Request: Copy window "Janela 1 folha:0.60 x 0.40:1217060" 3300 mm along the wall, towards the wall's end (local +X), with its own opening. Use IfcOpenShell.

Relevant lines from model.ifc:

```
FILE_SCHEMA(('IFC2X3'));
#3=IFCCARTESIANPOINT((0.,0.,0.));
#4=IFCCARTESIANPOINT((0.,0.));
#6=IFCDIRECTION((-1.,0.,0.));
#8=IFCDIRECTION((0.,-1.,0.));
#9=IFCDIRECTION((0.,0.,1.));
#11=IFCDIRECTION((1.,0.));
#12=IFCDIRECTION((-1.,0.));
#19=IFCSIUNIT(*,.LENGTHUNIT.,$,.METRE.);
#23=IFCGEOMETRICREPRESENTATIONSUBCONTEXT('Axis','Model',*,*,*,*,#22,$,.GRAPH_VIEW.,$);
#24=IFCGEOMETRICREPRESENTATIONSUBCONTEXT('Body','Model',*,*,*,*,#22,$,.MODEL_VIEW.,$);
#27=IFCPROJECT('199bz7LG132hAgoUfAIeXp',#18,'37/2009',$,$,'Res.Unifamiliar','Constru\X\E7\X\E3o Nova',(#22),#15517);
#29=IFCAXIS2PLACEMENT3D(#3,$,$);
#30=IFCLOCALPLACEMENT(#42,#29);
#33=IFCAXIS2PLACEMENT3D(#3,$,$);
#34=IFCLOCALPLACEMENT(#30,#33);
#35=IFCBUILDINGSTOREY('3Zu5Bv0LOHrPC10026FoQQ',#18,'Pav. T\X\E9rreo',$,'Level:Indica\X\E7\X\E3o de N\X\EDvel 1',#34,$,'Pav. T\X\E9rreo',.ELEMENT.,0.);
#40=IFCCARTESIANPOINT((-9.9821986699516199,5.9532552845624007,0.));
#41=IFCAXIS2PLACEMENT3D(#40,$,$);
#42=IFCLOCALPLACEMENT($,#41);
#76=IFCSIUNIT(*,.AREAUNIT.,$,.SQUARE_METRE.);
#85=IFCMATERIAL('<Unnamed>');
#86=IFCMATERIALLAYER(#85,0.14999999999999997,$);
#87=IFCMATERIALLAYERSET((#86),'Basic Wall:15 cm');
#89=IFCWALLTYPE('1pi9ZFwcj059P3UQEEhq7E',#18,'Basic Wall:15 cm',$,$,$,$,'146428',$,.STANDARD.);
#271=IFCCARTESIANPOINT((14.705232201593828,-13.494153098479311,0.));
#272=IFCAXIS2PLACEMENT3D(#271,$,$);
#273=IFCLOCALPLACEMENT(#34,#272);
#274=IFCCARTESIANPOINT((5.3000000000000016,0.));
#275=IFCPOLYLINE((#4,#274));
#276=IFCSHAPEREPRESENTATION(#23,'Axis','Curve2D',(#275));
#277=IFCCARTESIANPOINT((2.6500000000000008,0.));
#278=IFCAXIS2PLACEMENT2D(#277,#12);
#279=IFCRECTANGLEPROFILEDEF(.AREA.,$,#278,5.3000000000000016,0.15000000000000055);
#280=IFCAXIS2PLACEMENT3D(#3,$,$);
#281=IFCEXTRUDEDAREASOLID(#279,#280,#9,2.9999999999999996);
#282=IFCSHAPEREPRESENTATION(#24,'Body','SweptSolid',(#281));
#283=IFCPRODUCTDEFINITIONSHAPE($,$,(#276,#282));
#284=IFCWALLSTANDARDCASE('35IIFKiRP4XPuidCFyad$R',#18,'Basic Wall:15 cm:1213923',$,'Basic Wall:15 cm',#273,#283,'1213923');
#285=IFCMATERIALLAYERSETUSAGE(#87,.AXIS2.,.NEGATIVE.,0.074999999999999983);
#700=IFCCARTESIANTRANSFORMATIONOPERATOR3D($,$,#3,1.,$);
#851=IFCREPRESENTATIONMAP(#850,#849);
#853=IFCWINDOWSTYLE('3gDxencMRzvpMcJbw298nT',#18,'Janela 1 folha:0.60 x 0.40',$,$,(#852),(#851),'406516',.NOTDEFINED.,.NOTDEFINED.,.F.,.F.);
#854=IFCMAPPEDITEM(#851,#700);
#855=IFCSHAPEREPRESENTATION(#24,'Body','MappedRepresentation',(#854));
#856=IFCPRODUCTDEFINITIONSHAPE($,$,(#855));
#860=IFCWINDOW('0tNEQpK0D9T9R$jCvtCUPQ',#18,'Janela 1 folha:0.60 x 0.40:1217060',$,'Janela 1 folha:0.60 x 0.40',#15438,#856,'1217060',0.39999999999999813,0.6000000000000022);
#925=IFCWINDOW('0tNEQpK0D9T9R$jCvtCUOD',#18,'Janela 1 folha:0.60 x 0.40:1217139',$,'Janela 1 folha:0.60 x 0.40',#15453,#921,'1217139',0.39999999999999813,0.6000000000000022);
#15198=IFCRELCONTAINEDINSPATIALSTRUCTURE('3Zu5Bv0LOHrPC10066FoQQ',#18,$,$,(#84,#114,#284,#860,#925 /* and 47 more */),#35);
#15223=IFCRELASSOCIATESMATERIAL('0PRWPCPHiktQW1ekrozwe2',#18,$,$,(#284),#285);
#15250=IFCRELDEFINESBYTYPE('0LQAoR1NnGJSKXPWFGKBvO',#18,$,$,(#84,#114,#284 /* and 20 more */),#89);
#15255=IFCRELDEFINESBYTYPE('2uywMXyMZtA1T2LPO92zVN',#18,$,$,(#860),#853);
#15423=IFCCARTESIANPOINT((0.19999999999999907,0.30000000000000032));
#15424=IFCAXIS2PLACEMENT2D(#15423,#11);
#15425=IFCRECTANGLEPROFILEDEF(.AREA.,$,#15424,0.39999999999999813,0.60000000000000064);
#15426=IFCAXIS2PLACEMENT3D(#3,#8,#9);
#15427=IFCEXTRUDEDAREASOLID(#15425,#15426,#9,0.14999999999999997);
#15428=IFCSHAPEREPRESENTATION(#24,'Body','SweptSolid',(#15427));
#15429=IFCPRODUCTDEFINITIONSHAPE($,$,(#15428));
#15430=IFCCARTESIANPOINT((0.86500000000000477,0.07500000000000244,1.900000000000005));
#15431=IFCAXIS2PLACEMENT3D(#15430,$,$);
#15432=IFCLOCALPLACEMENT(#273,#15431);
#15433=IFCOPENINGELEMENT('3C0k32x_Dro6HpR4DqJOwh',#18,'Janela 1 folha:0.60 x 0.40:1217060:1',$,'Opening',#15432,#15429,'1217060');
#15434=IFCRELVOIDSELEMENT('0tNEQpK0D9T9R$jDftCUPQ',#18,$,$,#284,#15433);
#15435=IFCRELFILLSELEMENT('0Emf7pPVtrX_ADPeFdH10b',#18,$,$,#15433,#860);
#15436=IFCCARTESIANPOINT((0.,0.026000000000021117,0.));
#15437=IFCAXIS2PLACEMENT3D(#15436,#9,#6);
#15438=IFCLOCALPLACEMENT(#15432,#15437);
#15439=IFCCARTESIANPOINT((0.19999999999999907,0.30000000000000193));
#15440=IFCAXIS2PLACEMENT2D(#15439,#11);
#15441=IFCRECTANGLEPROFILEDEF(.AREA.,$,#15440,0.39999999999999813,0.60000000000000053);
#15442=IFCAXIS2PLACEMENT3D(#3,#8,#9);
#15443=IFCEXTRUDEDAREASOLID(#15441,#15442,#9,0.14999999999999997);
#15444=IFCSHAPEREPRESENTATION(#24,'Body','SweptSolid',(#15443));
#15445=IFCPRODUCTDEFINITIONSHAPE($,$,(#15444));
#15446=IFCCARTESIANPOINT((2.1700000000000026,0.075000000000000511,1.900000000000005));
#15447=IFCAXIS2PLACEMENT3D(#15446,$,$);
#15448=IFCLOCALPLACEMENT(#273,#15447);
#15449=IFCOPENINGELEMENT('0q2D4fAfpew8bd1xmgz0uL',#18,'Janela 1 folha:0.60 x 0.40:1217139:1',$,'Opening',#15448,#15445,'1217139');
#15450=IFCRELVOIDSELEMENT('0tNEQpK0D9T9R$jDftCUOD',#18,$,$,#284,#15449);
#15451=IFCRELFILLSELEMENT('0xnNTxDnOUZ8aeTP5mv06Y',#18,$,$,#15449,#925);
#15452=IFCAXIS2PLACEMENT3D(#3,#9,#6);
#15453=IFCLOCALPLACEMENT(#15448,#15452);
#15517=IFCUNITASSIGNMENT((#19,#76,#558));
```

```python
import ifcopenshell
import ifcopenshell.api.feature
import ifcopenshell.api.geometry
import ifcopenshell.api.root
import ifcopenshell.geom
import ifcopenshell.util.element
import ifcopenshell.util.placement
import ifcopenshell.util.shape

model = ifcopenshell.open("model.ifc")
settings = ifcopenshell.geom.settings()


def volume(element):
    """Net volume in cubic metres, openings subtracted."""
    shape = ifcopenshell.geom.create_shape(settings, element)
    return ifcopenshell.util.shape.get_volume(shape.geometry)


def reuse_history(source, copy):
    """copy_class also copies each property set's owner history, people and application; keep the originals."""
    for rel in copy.IsDefinedBy:
        if rel.is_a("IfcRelDefinesByProperties") and (history := rel.RelatingPropertyDefinition.OwnerHistory):
            rel.RelatingPropertyDefinition.OwnerHistory = source.OwnerHistory
            ifcopenshell.util.element.remove_deep2(model, history)


window = model.by_id(860)
opening = window.FillsVoids[0].RelatingOpeningElement
wall = opening.VoidsElements[0].RelatingBuildingElement
before = volume(wall)
shift = ifcopenshell.util.placement.get_local_placement(wall.ObjectPlacement)[:3, 0] * 3.3

# copy_class copies the void relationship, type, container and properties, but no geometry.
new_opening = ifcopenshell.api.root.copy_class(model, product=opening)
new_opening.Representation = ifcopenshell.util.element.copy_deep(
    model, opening.Representation, exclude=["IfcGeometricRepresentationContext", "IfcRepresentationMap"]
)
new_opening.Name = "Janela 1 folha:0.60 x 0.40"
new_opening.Tag = None
new_window = ifcopenshell.api.root.copy_class(model, product=window)
new_window.Representation = ifcopenshell.util.element.copy_deep(
    model, window.Representation, exclude=["IfcGeometricRepresentationContext", "IfcRepresentationMap"]
)
new_window.Name = "Janela 1 folha:0.60 x 0.40"
new_window.Tag = None
reuse_history(window, new_window)
fills = ifcopenshell.api.feature.add_filling(model, opening=new_opening, element=new_window)
fills.OwnerHistory = new_window.OwnerHistory  # required in IFC2X3

for old, new in ((opening, new_opening), (window, new_window)):
    matrix = ifcopenshell.util.placement.get_local_placement(old.ObjectPlacement)
    matrix[:3, 3] += shift
    ifcopenshell.api.geometry.edit_object_placement(model, product=new, matrix=matrix, is_si=False)

after = volume(wall)

print(f"wall volume {before:.3f} -> {after:.3f} m3")

model.write("model-out.ifc")
```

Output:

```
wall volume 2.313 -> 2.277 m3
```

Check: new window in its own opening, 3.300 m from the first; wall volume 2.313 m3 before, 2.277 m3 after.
